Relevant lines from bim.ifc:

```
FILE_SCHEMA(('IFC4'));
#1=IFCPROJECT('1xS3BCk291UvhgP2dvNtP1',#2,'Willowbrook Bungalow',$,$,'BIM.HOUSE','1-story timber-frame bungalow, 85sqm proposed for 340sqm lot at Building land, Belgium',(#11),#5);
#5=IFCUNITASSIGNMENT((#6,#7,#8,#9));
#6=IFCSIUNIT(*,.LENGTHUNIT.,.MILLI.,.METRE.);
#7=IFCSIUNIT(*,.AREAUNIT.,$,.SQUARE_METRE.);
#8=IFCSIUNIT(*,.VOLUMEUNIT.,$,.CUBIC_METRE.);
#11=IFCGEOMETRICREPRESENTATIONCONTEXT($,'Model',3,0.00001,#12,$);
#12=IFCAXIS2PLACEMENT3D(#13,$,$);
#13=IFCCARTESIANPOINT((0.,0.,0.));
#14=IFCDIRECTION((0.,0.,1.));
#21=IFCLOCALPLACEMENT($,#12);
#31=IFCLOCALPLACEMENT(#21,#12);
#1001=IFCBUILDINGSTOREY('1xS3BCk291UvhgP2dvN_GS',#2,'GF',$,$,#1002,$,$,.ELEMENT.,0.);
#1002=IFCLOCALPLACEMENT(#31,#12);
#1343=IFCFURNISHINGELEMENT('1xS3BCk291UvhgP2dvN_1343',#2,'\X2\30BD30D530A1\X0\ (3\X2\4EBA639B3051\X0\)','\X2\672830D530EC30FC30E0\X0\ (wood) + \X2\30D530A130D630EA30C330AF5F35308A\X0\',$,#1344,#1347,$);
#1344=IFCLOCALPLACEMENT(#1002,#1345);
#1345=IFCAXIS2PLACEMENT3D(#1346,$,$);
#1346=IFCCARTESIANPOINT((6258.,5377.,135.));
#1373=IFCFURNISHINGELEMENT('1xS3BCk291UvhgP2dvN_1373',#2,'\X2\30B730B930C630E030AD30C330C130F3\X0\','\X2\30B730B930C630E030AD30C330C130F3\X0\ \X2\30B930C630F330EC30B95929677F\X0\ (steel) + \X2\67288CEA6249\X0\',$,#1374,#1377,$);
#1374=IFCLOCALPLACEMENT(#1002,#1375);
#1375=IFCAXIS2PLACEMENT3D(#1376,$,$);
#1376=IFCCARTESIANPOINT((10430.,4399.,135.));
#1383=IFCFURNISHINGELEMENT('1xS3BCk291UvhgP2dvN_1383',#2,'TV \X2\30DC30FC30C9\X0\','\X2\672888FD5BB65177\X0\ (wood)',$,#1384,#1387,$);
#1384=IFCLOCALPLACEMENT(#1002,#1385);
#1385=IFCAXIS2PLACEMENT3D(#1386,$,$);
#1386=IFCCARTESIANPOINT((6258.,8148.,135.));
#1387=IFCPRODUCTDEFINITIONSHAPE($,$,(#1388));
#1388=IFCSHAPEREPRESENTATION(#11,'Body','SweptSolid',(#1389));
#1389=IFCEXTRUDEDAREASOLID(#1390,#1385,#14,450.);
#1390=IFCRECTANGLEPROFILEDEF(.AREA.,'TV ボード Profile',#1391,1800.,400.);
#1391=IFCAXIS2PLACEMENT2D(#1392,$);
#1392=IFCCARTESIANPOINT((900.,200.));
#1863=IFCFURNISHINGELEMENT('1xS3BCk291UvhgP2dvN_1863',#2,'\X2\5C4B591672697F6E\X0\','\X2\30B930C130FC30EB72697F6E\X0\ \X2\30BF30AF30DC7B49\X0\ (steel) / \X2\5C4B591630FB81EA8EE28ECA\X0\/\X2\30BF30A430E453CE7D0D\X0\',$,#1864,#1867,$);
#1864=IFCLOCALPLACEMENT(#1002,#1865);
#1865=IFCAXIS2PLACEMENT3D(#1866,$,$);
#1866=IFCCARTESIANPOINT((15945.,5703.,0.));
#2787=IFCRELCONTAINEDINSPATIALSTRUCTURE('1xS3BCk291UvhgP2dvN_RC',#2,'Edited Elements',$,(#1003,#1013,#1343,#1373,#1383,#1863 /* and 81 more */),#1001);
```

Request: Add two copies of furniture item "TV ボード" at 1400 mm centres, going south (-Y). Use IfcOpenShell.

```python
import numpy as np
import ifcopenshell
import ifcopenshell.api.geometry
import ifcopenshell.api.root
import ifcopenshell.util.element
import ifcopenshell.util.placement
import ifcopenshell.util.unit

model = ifcopenshell.open("bim.ifc")
unit_scale = ifcopenshell.util.unit.calculate_unit_scale(model)


def reuse_history(source, copy):
    """copy_class also copies each property set's owner history, people and application; keep the originals."""
    for rel in copy.IsDefinedBy:
        if rel.is_a("IfcRelDefinesByProperties") and (history := rel.RelatingPropertyDefinition.OwnerHistory):
            rel.RelatingPropertyDefinition.OwnerHistory = source.OwnerHistory
            ifcopenshell.util.element.remove_deep2(model, history)


source = model.by_id(1383)
base = ifcopenshell.util.placement.get_local_placement(source.ObjectPlacement)
step = np.array([0.0, -1.0, 0.0]) * 1.4 / unit_scale

for i in range(1, 3):
    copy = ifcopenshell.api.root.copy_class(model, product=source)
    copy.Representation = ifcopenshell.util.element.copy_deep(
        model, source.Representation, exclude=["IfcGeometricRepresentationContext", "IfcRepresentationMap"]
    )
    reuse_history(source, copy)
    matrix = base.copy()
    matrix[:3, 3] += i * step
    print("added at", matrix[:3, 3].round(3) + 0.0)
    ifcopenshell.api.geometry.edit_object_placement(model, product=copy, matrix=matrix, is_si=False)

model.write("bim_v2.ifc")
```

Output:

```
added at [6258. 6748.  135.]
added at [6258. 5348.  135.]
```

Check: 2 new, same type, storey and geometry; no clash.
